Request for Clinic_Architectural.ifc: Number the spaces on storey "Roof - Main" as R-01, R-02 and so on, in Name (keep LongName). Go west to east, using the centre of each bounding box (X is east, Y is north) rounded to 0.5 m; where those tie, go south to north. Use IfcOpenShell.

First a look at what the model holds.

```python
import ifcopenshell
import ifcopenshell.util.element
import ifcopenshell.util.placement

model = ifcopenshell.open("Clinic_Architectural.ifc")
print(model.schema)
storey = next(s for s in model.by_type("IfcBuildingStorey") if s.Name == "Roof - Main")
spaces = [e for e in ifcopenshell.util.element.get_decomposition(storey) if e.is_a("IfcSpace")]
for e in sorted(spaces, key=lambda e: e.id()):
    origin = ifcopenshell.util.placement.get_local_placement(e.ObjectPlacement)[:3, 3]
    print(e.id(), e.Name, e.LongName, origin.round(2) + 0.0, sep=" | ")
```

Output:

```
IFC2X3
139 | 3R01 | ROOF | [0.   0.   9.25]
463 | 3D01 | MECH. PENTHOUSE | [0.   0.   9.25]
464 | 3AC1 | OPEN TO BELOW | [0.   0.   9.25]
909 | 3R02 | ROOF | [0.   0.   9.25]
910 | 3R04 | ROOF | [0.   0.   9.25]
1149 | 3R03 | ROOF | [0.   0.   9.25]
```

```python
import ifcopenshell
import ifcopenshell.geom
import ifcopenshell.util.element
import ifcopenshell.util.shape

model = ifcopenshell.open("Clinic_Architectural.ifc")
settings = ifcopenshell.geom.settings()
settings.set("use-world-coords", True)


def centre(element):
    shape = ifcopenshell.geom.create_shape(settings, element)
    return ifcopenshell.util.shape.get_bbox_centroid(shape.geometry)


storey = next(s for s in model.by_type("IfcBuildingStorey") if s.Name == "Roof - Main")
spaces = [e for e in ifcopenshell.util.element.get_decomposition(storey) if e.is_a("IfcSpace")]

# Insertion points can sit at a corner or the storey origin, so sort by the geometry (in metres).
centres = {e: centre(e) for e in spaces}
spaces.sort(key=lambda e: (round(centres[e][0] / 0.5), centres[e][1]))

for i, e in enumerate(spaces, start=1):
    number = f"R-{i:02d}"
    e.Name = number
    print(e.id(), number)

model.write("Clinic_Architectural_edited.ifc")
```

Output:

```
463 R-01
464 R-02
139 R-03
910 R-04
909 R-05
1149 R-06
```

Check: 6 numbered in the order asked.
